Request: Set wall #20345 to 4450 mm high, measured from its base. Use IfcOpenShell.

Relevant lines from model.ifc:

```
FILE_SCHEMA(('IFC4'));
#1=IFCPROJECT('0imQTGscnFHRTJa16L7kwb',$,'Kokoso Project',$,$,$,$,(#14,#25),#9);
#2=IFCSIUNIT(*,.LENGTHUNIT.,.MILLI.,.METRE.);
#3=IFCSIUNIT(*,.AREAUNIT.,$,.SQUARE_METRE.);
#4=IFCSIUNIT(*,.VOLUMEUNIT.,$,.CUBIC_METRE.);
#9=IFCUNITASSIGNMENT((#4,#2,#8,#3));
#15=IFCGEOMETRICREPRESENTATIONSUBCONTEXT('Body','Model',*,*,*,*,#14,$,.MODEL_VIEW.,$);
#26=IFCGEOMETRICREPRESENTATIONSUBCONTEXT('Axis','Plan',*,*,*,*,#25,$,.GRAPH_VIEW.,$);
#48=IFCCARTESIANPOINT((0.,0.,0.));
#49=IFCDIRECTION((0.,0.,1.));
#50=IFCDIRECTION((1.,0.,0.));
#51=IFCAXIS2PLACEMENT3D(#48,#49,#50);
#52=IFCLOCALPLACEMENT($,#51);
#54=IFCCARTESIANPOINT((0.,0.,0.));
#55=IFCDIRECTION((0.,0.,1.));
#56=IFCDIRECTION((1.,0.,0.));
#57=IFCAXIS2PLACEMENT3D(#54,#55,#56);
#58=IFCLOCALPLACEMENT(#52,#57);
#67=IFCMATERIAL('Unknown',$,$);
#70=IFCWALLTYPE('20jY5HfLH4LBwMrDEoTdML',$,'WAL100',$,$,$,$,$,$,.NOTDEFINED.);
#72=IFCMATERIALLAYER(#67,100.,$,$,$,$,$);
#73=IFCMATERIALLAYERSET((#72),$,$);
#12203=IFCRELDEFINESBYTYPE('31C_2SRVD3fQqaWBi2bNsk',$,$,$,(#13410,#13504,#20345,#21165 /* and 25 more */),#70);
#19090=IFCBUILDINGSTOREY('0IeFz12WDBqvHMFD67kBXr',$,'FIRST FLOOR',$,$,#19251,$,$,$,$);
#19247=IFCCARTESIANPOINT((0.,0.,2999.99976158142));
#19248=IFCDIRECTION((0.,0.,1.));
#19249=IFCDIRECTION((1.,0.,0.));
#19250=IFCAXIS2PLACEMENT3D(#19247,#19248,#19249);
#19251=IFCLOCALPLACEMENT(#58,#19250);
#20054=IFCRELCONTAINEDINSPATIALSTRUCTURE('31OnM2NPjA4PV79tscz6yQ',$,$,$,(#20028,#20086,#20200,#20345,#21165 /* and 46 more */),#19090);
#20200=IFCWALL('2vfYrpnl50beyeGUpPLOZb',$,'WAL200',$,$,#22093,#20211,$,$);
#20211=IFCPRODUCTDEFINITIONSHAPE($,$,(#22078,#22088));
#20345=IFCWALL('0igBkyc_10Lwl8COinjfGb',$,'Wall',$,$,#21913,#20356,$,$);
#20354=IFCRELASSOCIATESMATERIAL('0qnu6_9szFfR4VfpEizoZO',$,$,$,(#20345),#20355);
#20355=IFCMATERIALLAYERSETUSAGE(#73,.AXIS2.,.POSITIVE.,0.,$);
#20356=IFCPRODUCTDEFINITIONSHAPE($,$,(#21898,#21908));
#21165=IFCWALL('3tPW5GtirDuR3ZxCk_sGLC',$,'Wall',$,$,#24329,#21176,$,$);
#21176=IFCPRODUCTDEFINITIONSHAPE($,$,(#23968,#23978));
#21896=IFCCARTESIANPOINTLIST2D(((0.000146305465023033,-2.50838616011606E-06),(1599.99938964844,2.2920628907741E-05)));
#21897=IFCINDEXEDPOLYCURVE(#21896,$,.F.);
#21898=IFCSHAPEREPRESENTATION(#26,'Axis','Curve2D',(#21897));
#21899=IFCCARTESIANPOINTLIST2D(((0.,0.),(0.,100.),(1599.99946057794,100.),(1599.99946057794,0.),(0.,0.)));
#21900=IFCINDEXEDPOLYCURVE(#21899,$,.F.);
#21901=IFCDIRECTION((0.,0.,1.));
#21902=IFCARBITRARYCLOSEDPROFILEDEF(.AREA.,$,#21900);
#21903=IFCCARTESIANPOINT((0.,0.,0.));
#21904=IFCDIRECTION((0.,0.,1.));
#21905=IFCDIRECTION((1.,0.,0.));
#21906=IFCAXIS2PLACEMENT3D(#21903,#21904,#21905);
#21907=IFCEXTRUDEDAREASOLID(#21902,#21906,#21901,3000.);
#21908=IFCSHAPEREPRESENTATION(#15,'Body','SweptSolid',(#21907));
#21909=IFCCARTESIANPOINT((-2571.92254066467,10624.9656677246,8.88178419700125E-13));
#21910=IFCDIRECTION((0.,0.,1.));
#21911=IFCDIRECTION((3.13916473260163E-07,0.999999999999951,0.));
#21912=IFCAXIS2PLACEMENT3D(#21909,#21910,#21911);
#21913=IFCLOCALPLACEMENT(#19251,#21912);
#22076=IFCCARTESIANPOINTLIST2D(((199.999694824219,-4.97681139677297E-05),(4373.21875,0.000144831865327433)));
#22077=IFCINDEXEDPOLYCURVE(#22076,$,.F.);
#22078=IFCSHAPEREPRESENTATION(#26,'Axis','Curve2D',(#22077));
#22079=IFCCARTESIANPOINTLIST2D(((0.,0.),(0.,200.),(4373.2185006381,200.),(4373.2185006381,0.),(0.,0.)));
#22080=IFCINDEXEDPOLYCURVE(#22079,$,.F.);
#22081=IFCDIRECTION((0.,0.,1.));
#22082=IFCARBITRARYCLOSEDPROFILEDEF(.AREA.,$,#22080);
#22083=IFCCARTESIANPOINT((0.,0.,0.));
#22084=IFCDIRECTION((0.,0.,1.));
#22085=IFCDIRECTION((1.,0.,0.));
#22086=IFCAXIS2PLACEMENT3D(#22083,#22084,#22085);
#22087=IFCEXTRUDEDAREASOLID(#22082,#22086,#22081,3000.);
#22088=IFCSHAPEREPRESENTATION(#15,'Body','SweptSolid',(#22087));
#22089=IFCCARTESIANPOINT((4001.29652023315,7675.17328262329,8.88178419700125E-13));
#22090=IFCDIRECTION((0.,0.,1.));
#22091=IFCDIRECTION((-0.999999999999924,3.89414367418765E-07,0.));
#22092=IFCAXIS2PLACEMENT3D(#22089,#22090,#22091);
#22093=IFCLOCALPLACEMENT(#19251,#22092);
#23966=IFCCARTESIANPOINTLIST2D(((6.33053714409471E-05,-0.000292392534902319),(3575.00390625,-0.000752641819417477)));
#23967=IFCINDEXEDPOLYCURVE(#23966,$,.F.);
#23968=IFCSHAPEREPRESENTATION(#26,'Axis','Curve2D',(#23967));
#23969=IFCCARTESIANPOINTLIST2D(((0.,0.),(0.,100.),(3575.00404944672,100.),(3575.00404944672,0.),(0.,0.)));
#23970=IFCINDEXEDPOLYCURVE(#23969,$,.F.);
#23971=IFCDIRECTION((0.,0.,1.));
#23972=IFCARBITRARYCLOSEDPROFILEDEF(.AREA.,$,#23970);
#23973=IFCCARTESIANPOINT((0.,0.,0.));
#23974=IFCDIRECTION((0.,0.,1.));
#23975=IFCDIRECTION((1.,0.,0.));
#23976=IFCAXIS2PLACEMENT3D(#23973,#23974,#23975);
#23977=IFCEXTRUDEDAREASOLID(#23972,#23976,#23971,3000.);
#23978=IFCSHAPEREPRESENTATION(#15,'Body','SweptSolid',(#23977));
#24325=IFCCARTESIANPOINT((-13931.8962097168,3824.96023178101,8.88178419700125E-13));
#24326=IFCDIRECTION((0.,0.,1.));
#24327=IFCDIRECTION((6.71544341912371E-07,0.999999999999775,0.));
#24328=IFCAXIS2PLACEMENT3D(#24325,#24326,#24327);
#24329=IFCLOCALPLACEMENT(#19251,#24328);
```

```python
import ifcopenshell
import ifcopenshell.geom
import ifcopenshell.util.representation
import ifcopenshell.util.shape
import ifcopenshell.util.unit

model = ifcopenshell.open("model.ifc")
unit_scale = ifcopenshell.util.unit.calculate_unit_scale(model)
settings = ifcopenshell.geom.settings()


def volume(element):
    """Net volume in cubic metres, openings subtracted."""
    shape = ifcopenshell.geom.create_shape(settings, element)
    return ifcopenshell.util.shape.get_volume(shape.geometry)


wall = model.by_guid("0igBkyc_10Lwl8COinjfGb")
before = volume(wall)

body = ifcopenshell.util.representation.get_representation(wall, "Model", "Body")
solid = body.Items[0]
old_height = solid.Depth
solid.Depth = 4.45 / unit_scale
after = volume(wall)

print(f"height {old_height:g} -> {solid.Depth:g}, volume {before:.3f} -> {after:.3f} m3")

model.write("model_updated.ifc")
```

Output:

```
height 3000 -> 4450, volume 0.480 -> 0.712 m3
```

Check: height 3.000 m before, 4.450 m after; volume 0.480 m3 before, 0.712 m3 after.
